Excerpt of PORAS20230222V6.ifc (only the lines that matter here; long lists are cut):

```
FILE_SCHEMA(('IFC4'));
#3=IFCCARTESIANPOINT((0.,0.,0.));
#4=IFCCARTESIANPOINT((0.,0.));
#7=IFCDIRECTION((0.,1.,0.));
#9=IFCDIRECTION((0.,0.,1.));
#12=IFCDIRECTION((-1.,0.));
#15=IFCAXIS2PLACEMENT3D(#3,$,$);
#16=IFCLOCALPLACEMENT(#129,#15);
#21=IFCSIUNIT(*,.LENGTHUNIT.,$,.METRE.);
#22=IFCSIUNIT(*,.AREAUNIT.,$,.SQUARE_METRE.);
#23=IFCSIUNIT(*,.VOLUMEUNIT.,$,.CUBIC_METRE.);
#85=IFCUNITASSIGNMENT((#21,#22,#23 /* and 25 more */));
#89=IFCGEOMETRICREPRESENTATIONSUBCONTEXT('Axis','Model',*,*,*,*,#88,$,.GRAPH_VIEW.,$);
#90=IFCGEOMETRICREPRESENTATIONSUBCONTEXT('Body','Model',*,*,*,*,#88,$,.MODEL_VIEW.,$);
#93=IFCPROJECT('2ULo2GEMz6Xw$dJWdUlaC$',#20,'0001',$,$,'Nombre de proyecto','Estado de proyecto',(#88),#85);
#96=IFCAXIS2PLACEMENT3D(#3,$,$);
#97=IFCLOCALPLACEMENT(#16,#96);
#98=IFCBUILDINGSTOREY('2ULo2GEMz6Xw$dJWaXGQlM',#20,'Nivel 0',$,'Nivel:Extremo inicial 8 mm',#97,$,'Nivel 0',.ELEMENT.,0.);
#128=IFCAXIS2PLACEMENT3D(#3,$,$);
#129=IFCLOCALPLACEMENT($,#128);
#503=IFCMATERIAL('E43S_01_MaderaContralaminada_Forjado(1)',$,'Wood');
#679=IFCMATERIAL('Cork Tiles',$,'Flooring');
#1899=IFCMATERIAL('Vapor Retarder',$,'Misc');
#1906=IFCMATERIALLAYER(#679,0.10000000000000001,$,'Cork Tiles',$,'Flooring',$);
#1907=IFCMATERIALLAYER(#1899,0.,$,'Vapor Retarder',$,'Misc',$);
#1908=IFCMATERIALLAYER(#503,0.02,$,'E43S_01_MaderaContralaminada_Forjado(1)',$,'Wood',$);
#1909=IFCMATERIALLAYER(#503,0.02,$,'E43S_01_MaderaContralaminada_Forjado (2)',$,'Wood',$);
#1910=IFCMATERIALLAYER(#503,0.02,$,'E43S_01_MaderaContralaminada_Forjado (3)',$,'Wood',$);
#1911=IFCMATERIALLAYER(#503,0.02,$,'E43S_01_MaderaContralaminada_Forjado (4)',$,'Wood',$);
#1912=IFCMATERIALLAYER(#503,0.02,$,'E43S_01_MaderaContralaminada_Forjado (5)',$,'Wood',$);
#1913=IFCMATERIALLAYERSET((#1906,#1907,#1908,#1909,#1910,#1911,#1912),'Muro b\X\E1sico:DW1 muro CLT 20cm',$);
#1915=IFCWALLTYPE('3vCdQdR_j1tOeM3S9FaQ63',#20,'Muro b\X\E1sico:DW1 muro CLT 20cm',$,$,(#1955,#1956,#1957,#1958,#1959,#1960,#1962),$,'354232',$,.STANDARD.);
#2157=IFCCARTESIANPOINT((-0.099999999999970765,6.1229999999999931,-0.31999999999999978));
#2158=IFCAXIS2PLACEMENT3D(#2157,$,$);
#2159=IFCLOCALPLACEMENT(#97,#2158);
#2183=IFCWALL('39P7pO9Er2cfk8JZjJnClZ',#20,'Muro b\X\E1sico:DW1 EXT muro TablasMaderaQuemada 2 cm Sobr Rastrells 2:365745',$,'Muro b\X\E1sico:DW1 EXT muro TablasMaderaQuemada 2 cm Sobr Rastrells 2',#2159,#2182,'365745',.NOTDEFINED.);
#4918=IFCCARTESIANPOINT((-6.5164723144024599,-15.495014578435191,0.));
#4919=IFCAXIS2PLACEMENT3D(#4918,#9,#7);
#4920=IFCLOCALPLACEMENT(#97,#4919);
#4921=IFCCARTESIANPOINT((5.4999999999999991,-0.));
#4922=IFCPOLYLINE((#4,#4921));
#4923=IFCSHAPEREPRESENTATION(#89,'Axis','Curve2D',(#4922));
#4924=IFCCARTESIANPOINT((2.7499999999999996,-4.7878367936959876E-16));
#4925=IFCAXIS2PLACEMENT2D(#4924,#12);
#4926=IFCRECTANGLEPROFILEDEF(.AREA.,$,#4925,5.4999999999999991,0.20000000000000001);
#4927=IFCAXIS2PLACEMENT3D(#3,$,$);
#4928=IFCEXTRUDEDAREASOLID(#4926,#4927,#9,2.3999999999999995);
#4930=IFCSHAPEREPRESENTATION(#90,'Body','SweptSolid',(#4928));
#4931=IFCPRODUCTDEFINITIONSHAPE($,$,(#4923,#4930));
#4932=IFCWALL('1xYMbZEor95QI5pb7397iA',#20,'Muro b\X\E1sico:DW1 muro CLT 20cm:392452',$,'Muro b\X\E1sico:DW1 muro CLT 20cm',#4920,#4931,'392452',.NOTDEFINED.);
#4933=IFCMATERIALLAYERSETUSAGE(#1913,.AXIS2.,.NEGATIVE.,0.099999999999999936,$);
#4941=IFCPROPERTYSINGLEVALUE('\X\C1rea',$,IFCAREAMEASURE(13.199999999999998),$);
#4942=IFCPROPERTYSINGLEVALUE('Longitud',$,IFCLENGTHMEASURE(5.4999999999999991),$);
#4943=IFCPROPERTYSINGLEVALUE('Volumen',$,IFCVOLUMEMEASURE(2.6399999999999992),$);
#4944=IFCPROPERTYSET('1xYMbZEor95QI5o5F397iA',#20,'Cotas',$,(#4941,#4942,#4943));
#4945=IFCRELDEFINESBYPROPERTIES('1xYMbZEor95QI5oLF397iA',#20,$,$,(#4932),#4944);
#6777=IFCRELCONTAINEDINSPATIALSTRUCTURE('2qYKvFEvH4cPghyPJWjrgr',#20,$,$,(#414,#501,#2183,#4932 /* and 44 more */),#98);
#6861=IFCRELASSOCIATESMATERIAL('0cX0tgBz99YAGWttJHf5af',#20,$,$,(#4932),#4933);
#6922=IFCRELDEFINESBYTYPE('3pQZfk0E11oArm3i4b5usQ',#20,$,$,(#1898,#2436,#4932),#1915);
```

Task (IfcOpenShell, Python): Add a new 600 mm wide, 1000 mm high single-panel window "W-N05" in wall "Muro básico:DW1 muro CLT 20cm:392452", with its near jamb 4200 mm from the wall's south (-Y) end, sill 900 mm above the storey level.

```python
import numpy as np
import ifcopenshell
import ifcopenshell.api.feature
import ifcopenshell.api.geometry
import ifcopenshell.api.pset
import ifcopenshell.api.root
import ifcopenshell.api.spatial
import ifcopenshell.geom
import ifcopenshell.util.element
import ifcopenshell.util.placement
import ifcopenshell.util.representation
import ifcopenshell.util.shape
import ifcopenshell.util.unit

model = ifcopenshell.open("PORAS20230222V6.ifc")
unit_scale = ifcopenshell.util.unit.calculate_unit_scale(model)
area_scale = ifcopenshell.util.unit.calculate_unit_scale(model, "AREAUNIT")
volume_scale = ifcopenshell.util.unit.calculate_unit_scale(model, "VOLUMEUNIT")
settings = ifcopenshell.geom.settings()


def volume(element):
    """Net volume in cubic metres, openings subtracted."""
    shape = ifcopenshell.geom.create_shape(settings, element)
    return ifcopenshell.util.shape.get_volume(shape.geometry)


wall = model.by_guid("1xYMbZEor95QI5pb7397iA")
storey = ifcopenshell.util.element.get_container(wall, ifc_class="IfcBuildingStorey")
context = ifcopenshell.util.representation.get_context(model, "Model", "Body", "MODEL_VIEW")
before = volume(wall)

width, height, from_end, sill = 0.6, 1, 4.2, 0.9  # metres

# The wall runs along its own X axis, and the end named is its -X end.
wall_shape = ifcopenshell.geom.create_shape(settings, wall)
x, y, z = ifcopenshell.util.shape.get_vertices(wall_shape.geometry).T
start = x.min() + from_end
face, thickness = float(y.min()), float(y.max() - y.min())
wall_matrix = ifcopenshell.util.placement.get_local_placement(wall.ObjectPlacement)
level = ifcopenshell.util.placement.get_local_placement(storey.ObjectPlacement)[2, 3]


def in_wall(x, y):
    """Placement at x, y metres in the wall's axes, at sill height."""
    matrix = wall_matrix.copy()
    matrix[:, 3] = wall_matrix @ np.array([x / unit_scale, y / unit_scale, 0.0, 1.0])
    matrix[2, 3] = level + sill / unit_scale
    return matrix


# Opening: a box that overshoots both wall faces by 50 mm.
opening = ifcopenshell.api.root.create_entity(model, ifc_class="IfcOpeningElement", predefined_type="OPENING")
box = ifcopenshell.api.geometry.add_wall_representation(
    model, context=context, length=width, height=height, thickness=thickness + 0.1
)
ifcopenshell.api.geometry.assign_representation(model, product=opening, representation=box)
ifcopenshell.api.geometry.edit_object_placement(model, product=opening, matrix=in_wall(start, face - 0.05), is_si=False)
ifcopenshell.api.feature.add_feature(model, feature=opening, element=wall)

window = ifcopenshell.api.root.create_entity(model, ifc_class="IfcWindow", name="W-N05", predefined_type="WINDOW")
window.OverallWidth, window.OverallHeight = width / unit_scale, height / unit_scale
window.PartitioningType = "SINGLE_PANEL"
body = ifcopenshell.api.geometry.add_window_representation(
    model,
    context=context,
    overall_width=window.OverallWidth,
    overall_height=window.OverallHeight,
    partition_type="SINGLE_PANEL",
)
ifcopenshell.api.geometry.assign_representation(model, product=window, representation=body)
ifcopenshell.api.spatial.assign_container(model, products=[window], relating_structure=storey)
ifcopenshell.api.feature.add_filling(model, opening=opening, element=window)

# Centre the window in the wall's thickness.
ifcopenshell.api.geometry.edit_object_placement(model, product=window, matrix=in_wall(start, face), is_si=False)
window_shape = ifcopenshell.geom.create_shape(settings, window)
depth = ifcopenshell.util.shape.get_vertices(window_shape.geometry)[:, 1]
offset = face + thickness / 2 - (depth.min() + depth.max()) / 2
ifcopenshell.api.geometry.edit_object_placement(model, product=window, matrix=in_wall(start, offset), is_si=False)

after = volume(wall)

# Update the wall's stored quantities.
pset = model.by_id(ifcopenshell.util.element.get_pset(wall, "Cotas", should_inherit=False)["id"])
ifcopenshell.api.pset.edit_pset(model, pset=pset, properties={
    "Área": model.create_entity("IfcAreaMeasure", after / thickness / area_scale),
    "Volumen": model.create_entity("IfcVolumeMeasure", after / volume_scale),
})

print(f"wall volume {before:.3f} -> {after:.3f} m3")

model.write("PORAS20230222V6_v2.ifc")
```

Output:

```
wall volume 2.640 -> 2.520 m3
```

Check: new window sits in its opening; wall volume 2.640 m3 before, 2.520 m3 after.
